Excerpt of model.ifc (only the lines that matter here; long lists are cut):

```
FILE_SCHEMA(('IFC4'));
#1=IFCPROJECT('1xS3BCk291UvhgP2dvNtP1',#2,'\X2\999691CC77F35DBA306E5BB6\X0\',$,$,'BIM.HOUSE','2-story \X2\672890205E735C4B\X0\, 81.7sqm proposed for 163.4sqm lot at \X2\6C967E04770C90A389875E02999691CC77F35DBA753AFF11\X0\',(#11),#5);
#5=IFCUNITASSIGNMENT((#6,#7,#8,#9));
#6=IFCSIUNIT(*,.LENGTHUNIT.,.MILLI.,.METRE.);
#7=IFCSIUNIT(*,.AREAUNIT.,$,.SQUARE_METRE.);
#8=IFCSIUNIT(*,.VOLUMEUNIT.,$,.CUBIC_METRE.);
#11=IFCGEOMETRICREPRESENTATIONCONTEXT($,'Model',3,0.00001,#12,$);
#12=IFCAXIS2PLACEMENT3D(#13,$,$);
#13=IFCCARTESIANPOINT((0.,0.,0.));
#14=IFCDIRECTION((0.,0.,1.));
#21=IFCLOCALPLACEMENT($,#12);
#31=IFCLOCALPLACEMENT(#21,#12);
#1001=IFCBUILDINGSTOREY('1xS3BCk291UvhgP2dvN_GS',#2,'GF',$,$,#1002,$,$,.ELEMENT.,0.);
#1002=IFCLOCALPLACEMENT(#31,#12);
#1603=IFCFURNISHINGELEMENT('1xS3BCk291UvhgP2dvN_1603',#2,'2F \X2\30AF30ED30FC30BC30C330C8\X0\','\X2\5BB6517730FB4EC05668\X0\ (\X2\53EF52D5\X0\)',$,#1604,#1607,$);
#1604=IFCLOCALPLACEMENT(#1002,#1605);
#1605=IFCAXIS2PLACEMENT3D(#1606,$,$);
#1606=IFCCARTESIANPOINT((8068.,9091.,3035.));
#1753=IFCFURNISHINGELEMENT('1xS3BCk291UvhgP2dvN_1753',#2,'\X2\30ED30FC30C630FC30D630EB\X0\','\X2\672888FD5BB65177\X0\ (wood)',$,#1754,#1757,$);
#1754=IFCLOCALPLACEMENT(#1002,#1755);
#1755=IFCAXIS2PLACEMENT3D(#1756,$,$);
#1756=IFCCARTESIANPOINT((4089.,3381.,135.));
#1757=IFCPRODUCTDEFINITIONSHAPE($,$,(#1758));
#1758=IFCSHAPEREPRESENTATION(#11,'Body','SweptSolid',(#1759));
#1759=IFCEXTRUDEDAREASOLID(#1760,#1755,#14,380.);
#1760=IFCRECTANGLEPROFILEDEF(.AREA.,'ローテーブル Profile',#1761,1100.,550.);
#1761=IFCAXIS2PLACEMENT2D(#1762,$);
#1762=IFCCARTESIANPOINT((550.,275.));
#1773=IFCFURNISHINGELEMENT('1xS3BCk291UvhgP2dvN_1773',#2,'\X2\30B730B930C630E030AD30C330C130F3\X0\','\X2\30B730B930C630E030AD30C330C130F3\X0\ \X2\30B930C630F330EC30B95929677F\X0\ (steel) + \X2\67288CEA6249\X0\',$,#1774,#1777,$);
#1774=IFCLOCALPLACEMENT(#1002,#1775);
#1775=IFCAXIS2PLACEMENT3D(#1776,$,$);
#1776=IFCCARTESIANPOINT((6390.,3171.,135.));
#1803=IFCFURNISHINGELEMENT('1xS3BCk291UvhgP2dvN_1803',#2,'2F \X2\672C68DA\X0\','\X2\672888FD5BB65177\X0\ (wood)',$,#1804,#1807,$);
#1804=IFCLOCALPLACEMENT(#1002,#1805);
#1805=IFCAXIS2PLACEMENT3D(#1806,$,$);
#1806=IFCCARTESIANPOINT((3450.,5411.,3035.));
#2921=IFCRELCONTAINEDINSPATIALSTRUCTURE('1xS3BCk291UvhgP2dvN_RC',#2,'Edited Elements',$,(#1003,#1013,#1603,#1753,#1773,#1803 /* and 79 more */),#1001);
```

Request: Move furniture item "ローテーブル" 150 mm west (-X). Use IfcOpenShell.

```python
import ifcopenshell
import ifcopenshell.api.geometry
import ifcopenshell.util.placement
import ifcopenshell.util.unit

model = ifcopenshell.open("model.ifc")
unit_scale = ifcopenshell.util.unit.calculate_unit_scale(model)

item = model.by_id(1753)
matrix = ifcopenshell.util.placement.get_local_placement(item.ObjectPlacement)
matrix[0, 3] -= 0.15 / unit_scale
ifcopenshell.api.geometry.edit_object_placement(model, product=item, matrix=matrix, is_si=False)

print(ifcopenshell.util.placement.get_local_placement(item.ObjectPlacement).round(3) + 0.0)

model.write("model-out.ifc")
```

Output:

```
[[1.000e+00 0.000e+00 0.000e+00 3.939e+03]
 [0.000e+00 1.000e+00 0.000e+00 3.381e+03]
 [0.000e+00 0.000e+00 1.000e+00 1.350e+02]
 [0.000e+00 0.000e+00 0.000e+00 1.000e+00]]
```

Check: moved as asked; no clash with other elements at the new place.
